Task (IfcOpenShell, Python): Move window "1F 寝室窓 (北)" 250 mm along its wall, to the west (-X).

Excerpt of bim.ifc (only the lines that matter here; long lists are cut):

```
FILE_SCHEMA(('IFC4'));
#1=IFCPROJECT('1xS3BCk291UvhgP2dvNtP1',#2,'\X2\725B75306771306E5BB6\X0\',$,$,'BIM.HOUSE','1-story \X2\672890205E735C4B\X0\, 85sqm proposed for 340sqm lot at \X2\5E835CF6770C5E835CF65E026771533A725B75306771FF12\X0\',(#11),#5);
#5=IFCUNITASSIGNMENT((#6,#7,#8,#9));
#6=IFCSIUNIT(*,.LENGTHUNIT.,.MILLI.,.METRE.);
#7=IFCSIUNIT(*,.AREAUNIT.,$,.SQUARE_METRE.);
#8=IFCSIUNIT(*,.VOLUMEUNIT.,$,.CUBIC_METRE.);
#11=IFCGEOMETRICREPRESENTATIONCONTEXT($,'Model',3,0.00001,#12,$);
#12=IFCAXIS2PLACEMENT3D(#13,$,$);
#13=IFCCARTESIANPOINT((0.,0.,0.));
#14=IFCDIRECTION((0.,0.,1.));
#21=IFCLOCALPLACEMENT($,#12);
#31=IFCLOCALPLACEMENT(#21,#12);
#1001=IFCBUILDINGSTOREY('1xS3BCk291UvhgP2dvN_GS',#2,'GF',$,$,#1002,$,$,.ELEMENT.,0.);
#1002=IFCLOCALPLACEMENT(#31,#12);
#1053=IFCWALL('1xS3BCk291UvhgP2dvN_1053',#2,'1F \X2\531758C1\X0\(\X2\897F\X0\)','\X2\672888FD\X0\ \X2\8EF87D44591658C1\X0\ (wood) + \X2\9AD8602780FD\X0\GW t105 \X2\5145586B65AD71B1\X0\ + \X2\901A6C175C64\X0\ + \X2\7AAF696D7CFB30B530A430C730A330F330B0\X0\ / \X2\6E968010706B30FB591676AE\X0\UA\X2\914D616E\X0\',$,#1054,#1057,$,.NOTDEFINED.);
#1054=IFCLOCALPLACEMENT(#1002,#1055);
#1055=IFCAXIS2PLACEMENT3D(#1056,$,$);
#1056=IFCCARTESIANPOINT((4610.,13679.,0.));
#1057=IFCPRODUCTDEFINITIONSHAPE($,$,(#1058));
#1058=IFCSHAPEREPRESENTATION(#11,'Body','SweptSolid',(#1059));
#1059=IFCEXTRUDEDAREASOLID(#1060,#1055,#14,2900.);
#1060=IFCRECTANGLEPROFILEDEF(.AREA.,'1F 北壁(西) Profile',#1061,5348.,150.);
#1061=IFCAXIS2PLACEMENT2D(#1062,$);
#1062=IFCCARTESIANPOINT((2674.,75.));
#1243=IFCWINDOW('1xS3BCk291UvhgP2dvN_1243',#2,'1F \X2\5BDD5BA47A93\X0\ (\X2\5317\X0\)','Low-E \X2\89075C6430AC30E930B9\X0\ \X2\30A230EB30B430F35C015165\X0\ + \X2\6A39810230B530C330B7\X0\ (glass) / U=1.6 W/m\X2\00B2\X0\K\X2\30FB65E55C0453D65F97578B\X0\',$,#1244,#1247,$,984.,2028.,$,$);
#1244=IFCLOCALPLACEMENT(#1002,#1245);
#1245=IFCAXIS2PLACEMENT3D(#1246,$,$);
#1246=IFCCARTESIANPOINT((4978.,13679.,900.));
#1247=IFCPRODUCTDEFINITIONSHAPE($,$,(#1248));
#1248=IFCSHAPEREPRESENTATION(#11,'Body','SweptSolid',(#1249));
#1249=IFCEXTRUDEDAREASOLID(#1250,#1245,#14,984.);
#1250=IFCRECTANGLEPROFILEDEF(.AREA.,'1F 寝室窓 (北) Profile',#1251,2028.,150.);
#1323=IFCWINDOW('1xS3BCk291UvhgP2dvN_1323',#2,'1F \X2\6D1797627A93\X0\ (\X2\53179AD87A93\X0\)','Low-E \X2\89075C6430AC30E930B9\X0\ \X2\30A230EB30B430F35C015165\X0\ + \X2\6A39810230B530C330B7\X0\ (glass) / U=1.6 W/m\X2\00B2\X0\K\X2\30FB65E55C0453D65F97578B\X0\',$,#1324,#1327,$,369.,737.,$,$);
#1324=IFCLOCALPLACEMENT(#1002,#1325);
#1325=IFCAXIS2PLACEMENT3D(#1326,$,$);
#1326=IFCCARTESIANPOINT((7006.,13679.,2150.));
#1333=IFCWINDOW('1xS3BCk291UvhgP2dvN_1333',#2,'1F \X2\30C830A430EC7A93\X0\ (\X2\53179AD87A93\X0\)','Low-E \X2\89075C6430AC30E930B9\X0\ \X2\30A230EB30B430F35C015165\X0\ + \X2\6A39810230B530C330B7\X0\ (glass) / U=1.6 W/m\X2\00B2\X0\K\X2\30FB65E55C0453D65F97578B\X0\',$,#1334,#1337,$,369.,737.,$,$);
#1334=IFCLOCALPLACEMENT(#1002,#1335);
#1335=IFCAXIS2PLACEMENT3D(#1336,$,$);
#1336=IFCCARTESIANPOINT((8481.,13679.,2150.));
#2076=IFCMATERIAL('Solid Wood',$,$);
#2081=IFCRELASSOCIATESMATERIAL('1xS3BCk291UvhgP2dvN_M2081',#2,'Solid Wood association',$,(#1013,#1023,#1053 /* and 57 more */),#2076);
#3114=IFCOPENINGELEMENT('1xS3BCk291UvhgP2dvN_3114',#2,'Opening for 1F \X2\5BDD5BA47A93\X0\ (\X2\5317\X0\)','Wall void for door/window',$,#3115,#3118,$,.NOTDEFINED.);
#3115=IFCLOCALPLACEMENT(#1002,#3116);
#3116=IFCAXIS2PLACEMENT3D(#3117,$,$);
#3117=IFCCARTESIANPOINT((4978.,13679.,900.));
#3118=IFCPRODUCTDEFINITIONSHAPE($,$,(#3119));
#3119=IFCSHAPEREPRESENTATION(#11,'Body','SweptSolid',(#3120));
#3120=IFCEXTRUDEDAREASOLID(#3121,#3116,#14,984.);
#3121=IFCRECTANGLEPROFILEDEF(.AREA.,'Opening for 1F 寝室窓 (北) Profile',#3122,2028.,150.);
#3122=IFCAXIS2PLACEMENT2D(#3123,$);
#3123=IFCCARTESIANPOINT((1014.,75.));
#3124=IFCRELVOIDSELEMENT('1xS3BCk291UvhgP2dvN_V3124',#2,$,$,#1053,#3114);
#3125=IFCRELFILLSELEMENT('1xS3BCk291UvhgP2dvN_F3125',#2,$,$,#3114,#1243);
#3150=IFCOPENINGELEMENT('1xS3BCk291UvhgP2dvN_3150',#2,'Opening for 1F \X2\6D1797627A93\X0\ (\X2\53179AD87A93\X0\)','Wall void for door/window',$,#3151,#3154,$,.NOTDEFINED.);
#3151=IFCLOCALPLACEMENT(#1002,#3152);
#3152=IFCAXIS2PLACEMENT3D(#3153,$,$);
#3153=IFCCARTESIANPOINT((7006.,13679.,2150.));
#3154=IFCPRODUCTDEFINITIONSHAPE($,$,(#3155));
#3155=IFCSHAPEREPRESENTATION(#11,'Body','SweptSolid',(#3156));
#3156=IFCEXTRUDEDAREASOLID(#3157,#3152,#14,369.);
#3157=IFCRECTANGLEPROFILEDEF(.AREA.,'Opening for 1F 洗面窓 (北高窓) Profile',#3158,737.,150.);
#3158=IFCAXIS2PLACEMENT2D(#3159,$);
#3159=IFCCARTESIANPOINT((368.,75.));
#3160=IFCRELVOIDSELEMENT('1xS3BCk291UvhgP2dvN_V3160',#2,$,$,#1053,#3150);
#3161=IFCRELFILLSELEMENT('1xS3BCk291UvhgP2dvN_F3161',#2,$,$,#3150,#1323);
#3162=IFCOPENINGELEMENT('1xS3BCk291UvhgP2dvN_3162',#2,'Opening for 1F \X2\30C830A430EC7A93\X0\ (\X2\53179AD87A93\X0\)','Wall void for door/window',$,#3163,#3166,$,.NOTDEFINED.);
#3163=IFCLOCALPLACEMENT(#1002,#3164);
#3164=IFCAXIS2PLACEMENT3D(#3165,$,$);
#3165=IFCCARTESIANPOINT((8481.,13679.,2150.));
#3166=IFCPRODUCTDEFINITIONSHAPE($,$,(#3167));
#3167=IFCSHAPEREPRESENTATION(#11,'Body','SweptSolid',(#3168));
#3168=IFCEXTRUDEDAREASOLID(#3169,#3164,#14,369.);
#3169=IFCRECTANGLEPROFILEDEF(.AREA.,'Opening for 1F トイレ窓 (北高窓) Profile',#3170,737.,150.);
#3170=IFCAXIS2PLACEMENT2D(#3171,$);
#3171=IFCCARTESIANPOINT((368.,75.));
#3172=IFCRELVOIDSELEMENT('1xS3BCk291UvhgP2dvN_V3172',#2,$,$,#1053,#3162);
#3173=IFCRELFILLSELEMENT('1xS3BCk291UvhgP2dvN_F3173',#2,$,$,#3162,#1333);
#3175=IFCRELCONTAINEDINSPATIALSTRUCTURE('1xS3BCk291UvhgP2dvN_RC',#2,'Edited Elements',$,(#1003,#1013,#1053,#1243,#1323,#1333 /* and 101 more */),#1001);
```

```python
import ifcopenshell
import ifcopenshell.api.geometry
import ifcopenshell.util.placement
import ifcopenshell.util.unit

model = ifcopenshell.open("bim.ifc")
unit_scale = ifcopenshell.util.unit.calculate_unit_scale(model)

window = model.by_guid("1xS3BCk291UvhgP2dvN_1243")
opening = window.FillsVoids[0].RelatingOpeningElement
wall = opening.VoidsElements[0].RelatingBuildingElement

wall_matrix = ifcopenshell.util.placement.get_local_placement(wall.ObjectPlacement)
shift = wall_matrix[:3, 0] * -0.25 / unit_scale
before = ifcopenshell.util.placement.get_local_placement(window.ObjectPlacement)[:3, 3].copy()

# The window is not placed relative to its opening, so move both.
for product in (opening, window):
    matrix = ifcopenshell.util.placement.get_local_placement(product.ObjectPlacement)
    matrix[:3, 3] += shift
    ifcopenshell.api.geometry.edit_object_placement(model, product=product, matrix=matrix, is_si=False)

after = ifcopenshell.util.placement.get_local_placement(window.ObjectPlacement)[:3, 3]
print("window moved by", (after - before).round(3) + 0.0)

model.write("bim_rev.ifc")
```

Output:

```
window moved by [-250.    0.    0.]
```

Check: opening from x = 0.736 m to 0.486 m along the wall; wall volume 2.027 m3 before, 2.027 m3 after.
